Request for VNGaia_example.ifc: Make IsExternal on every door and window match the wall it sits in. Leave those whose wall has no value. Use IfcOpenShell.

First a look at what the model holds.

```python
import ifcopenshell
import ifcopenshell.util.element

model = ifcopenshell.open("VNGaia_example.ifc")
print(model.schema)
seen = {}
for e in model.by_type("IfcDoor") + model.by_type("IfcWindow"):
    if not e.FillsVoids:
        continue
    host = e.FillsVoids[0].RelatingOpeningElement.VoidsElements[0].RelatingBuildingElement
    own = ifcopenshell.util.element.get_pset(e, f"Pset_{e.is_a()[3:].removesuffix('StandardCase')}Common", "IsExternal")
    wall = ifcopenshell.util.element.get_pset(host, "Pset_WallCommon", "IsExternal")
    seen[e.is_a(), own, wall] = seen.get((e.is_a(), own, wall), 0) + 1
for (cls, own, wall), count in sorted(seen.items(), key=str):
    print(count, cls, "IsExternal:", own, "| host wall:", wall)
```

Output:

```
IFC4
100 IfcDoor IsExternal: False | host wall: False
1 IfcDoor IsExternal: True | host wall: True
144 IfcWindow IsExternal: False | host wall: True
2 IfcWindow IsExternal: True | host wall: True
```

```python
import ifcopenshell
import ifcopenshell.api.pset
import ifcopenshell.util.element

model = ifcopenshell.open("VNGaia_example.ifc")

count = 0
for ifc_class, pset_name in (("IfcDoor", "Pset_DoorCommon"), ("IfcWindow", "Pset_WindowCommon")):
    for e in model.by_type(ifc_class):
        if not e.FillsVoids:
            continue
        host = e.FillsVoids[0].RelatingOpeningElement.VoidsElements[0].RelatingBuildingElement
        external = ifcopenshell.util.element.get_pset(host, "Pset_WallCommon", "IsExternal")
        if external is None or ifcopenshell.util.element.get_pset(e, pset_name, "IsExternal") == external:
            continue
        pset = ifcopenshell.api.pset.add_pset(model, product=e, name=pset_name)
        ifcopenshell.api.pset.edit_pset(model, pset=pset, properties={"IsExternal": external})
        count += 1

print(count, "updated")

model.write("VNGaia_example_v2.ifc")
```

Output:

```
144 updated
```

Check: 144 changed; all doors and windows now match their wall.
